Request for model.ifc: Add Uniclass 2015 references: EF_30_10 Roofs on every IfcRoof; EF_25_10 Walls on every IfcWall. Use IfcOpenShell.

First a look at what the model holds.

```python
import ifcopenshell

model = ifcopenshell.open("model.ifc")
print(model.schema)
print("classifications:", [c.Name for c in model.by_type("IfcClassification")])
for ifc_class in ("IfcDoor", "IfcRoof", "IfcStair", "IfcWall", "IfcWindow"):
    print(ifc_class, len(model.by_type(ifc_class)))
```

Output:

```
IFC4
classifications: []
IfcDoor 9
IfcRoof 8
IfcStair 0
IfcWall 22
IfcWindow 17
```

```python
import ifcopenshell
import ifcopenshell.api.classification

model = ifcopenshell.open("model.ifc")

system = ifcopenshell.api.classification.add_classification(model, classification="Uniclass 2015")

codes = {
    "IfcRoof": ("EF_30_10", "Roofs"),
    "IfcWall": ("EF_25_10", "Walls"),
}
for ifc_class, (code, name) in codes.items():
    products = model.by_type(ifc_class)
    ifcopenshell.api.classification.add_reference(
        model, products=products, classification=system, identification=code, name=name
    )
    print(code, len(products))

model.write("model_updated.ifc")
```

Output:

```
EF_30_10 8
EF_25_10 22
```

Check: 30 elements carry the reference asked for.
